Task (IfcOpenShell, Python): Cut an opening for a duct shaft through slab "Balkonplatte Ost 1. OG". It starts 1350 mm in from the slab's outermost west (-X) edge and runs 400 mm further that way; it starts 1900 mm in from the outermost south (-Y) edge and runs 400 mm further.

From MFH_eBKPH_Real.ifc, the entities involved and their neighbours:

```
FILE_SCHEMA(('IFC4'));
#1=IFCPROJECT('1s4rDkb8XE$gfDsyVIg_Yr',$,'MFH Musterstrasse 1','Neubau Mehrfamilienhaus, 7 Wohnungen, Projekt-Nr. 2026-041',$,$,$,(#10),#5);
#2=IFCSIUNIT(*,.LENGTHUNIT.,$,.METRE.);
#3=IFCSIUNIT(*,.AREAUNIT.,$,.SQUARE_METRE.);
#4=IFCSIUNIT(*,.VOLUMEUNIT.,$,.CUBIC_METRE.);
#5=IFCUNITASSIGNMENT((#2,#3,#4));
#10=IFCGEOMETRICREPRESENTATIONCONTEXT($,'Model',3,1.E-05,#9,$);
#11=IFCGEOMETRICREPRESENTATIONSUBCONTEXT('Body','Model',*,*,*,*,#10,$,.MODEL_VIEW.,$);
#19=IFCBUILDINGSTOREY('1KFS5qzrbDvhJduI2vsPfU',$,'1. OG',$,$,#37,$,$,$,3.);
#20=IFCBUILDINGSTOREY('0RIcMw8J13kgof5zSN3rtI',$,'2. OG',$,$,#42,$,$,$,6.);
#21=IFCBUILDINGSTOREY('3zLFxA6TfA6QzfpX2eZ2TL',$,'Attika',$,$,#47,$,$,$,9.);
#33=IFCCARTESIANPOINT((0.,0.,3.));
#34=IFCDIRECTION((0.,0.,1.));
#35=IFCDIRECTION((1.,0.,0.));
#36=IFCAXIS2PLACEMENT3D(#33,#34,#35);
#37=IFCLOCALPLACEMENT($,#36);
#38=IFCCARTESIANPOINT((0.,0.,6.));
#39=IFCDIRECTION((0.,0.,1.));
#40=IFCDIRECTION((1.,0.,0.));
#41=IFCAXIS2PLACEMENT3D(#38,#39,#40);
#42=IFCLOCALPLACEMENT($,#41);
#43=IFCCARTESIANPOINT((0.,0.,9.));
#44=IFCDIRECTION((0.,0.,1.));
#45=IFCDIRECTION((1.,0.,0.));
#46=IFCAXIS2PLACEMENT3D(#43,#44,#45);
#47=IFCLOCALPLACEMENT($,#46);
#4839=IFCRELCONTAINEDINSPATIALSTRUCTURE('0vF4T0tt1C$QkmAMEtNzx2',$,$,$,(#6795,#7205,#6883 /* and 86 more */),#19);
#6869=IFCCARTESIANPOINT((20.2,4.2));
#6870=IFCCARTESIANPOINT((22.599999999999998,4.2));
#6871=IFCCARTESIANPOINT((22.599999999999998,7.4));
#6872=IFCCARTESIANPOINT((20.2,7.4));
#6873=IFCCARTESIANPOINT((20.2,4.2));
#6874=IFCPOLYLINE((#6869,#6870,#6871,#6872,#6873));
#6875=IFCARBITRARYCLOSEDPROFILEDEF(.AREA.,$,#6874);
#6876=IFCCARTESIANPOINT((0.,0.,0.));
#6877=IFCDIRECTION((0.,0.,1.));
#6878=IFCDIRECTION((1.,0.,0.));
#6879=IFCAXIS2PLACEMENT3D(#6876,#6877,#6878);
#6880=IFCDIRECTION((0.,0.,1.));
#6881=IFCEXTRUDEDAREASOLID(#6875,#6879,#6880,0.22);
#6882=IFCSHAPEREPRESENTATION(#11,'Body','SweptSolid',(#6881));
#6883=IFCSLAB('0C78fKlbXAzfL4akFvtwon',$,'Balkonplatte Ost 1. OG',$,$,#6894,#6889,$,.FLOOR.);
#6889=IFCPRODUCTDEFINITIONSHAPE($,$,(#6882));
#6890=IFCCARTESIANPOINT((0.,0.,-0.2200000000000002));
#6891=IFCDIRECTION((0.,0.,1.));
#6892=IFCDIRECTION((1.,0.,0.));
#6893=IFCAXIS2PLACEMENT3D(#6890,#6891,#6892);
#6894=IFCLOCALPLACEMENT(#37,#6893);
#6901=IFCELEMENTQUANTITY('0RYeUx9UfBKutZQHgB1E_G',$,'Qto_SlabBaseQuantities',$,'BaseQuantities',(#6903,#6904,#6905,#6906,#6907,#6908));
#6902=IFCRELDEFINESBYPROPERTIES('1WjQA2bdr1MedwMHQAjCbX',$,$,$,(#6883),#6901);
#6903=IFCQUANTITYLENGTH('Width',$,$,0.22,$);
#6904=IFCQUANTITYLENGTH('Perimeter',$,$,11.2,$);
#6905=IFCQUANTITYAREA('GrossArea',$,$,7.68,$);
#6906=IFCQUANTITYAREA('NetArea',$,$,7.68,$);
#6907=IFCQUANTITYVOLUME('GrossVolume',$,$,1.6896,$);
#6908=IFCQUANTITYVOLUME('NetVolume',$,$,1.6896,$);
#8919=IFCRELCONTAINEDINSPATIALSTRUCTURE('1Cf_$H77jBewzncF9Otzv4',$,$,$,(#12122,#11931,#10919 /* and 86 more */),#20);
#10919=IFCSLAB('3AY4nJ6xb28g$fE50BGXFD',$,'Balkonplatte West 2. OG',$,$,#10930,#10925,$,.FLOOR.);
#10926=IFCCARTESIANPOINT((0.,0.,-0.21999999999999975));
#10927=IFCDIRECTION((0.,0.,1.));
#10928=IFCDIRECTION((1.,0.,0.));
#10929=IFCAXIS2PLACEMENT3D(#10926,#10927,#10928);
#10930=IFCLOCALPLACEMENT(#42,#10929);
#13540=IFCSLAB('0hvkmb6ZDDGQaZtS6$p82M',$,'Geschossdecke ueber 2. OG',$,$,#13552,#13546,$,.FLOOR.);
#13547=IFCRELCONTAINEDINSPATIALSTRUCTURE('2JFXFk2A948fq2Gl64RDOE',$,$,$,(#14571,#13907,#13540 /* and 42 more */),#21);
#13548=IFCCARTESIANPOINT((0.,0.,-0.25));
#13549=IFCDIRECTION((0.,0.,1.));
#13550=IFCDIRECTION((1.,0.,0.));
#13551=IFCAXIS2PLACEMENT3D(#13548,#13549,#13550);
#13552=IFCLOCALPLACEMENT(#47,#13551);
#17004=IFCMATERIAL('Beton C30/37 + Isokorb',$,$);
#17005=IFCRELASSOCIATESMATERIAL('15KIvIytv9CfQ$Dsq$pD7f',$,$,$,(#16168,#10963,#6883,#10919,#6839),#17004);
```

```python
import numpy as np
import ifcopenshell
import ifcopenshell.api.feature
import ifcopenshell.api.geometry
import ifcopenshell.api.pset
import ifcopenshell.api.root
import ifcopenshell.geom
import ifcopenshell.util.element
import ifcopenshell.util.placement
import ifcopenshell.util.representation
import ifcopenshell.util.shape
import ifcopenshell.util.unit

model = ifcopenshell.open("MFH_eBKPH_Real.ifc")
unit_scale = ifcopenshell.util.unit.calculate_unit_scale(model)
area_scale = ifcopenshell.util.unit.calculate_unit_scale(model, "AREAUNIT")
volume_scale = ifcopenshell.util.unit.calculate_unit_scale(model, "VOLUMEUNIT")
settings = ifcopenshell.geom.settings()


def volume(element):
    """Net volume in cubic metres, openings subtracted."""
    shape = ifcopenshell.geom.create_shape(settings, element)
    return ifcopenshell.util.shape.get_volume(shape.geometry)


slab = model.by_id(6883)
before = volume(slab)

# Extent in the slab's own axes, in metres. The edges named are its -X and -Y sides.
slab_shape = ifcopenshell.geom.create_shape(settings, slab)
vertices = ifcopenshell.util.shape.get_vertices(slab_shape.geometry)
x_min, y_min, bottom = vertices.min(axis=0)
top = vertices[:, 2].max()

opening = ifcopenshell.api.root.create_entity(model, ifc_class="IfcOpeningElement", name="Duct shaft opening", predefined_type="OPENING")
context = ifcopenshell.util.representation.get_context(model, "Model", "Body", "MODEL_VIEW")
width, depth = 0.4, 0.4
outline = [(0.0, 0.0), (width, 0.0), (width, depth), (0.0, depth), (0.0, 0.0)]
# Overshoot both faces by 50 mm so the cut is clean.
shape = ifcopenshell.api.geometry.add_slab_representation(
    model, context=context, depth=top - bottom + 0.1, polyline=outline
)
ifcopenshell.api.geometry.assign_representation(model, product=opening, representation=shape)

matrix = ifcopenshell.util.placement.get_local_placement(slab.ObjectPlacement)
matrix[:, 3] = matrix @ np.append(np.array([x_min + 1.35, y_min + 1.9, bottom - 0.05]) / unit_scale, 1.0)
ifcopenshell.api.geometry.edit_object_placement(model, product=opening, matrix=matrix, is_si=False)
ifcopenshell.api.feature.add_feature(model, feature=opening, element=slab)

after = volume(slab)

# Update the slab's stored quantities.
qto = model.by_id(ifcopenshell.util.element.get_pset(slab, "Qto_SlabBaseQuantities", should_inherit=False)["id"])
ifcopenshell.api.pset.edit_qto(model, qto=qto, properties={
    "NetArea": after / (top - bottom) / area_scale,
    "NetVolume": after / volume_scale,
})

print(f"slab volume {before:.3f} -> {after:.3f} m3")

model.write("MFH_eBKPH_Real_updated.ifc")
```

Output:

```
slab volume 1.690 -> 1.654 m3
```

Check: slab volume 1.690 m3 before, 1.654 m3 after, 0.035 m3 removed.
